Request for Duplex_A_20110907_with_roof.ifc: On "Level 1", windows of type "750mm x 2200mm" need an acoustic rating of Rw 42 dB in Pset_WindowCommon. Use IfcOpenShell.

First a look at what the model holds.

```python
import ifcopenshell
import ifcopenshell.util.element

model = ifcopenshell.open("Duplex_A_20110907_with_roof.ifc")
print(model.schema)
storey = next(s for s in model.by_type("IfcBuildingStorey") if s.Name == "Level 1")
windows = [e for e in ifcopenshell.util.element.get_decomposition(storey) if e.is_a("IfcWindow")]
seen = {}
for e in windows:
    element_type = ifcopenshell.util.element.get_type(e)
    key = (element_type.Name if element_type != e and element_type else None, ifcopenshell.util.element.get_pset(e, "Pset_WindowCommon", "AcousticRating"))
    seen[key] = seen.get(key, 0) + 1
for (name, value), count in sorted(seen.items(), key=str):
    print(count, "x", name, "|", value)
```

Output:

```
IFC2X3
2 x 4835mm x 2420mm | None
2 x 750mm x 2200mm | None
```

```python
import ifcopenshell
import ifcopenshell.api.pset
import ifcopenshell.util.element

model = ifcopenshell.open("Duplex_A_20110907_with_roof.ifc")

storey = next(s for s in model.by_type("IfcBuildingStorey") if s.Name == "Level 1")
windows = [e for e in ifcopenshell.util.element.get_decomposition(storey) if e.is_a("IfcWindow")]

count = 0
for e in windows:
    element_type = ifcopenshell.util.element.get_type(e)
    if element_type in (None, e) or element_type.Name != "750mm x 2200mm":
        continue
    # add_pset returns the element's existing set when there is one.
    pset = ifcopenshell.api.pset.add_pset(model, product=e, name="Pset_WindowCommon")
    ifcopenshell.api.pset.edit_pset(model, pset=pset, properties={"AcousticRating": "Rw 42 dB"})
    count += 1

print(count, "windows updated")

model.write("Duplex_A_20110907_with_roof_edited.ifc")
```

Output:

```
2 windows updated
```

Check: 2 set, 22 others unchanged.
